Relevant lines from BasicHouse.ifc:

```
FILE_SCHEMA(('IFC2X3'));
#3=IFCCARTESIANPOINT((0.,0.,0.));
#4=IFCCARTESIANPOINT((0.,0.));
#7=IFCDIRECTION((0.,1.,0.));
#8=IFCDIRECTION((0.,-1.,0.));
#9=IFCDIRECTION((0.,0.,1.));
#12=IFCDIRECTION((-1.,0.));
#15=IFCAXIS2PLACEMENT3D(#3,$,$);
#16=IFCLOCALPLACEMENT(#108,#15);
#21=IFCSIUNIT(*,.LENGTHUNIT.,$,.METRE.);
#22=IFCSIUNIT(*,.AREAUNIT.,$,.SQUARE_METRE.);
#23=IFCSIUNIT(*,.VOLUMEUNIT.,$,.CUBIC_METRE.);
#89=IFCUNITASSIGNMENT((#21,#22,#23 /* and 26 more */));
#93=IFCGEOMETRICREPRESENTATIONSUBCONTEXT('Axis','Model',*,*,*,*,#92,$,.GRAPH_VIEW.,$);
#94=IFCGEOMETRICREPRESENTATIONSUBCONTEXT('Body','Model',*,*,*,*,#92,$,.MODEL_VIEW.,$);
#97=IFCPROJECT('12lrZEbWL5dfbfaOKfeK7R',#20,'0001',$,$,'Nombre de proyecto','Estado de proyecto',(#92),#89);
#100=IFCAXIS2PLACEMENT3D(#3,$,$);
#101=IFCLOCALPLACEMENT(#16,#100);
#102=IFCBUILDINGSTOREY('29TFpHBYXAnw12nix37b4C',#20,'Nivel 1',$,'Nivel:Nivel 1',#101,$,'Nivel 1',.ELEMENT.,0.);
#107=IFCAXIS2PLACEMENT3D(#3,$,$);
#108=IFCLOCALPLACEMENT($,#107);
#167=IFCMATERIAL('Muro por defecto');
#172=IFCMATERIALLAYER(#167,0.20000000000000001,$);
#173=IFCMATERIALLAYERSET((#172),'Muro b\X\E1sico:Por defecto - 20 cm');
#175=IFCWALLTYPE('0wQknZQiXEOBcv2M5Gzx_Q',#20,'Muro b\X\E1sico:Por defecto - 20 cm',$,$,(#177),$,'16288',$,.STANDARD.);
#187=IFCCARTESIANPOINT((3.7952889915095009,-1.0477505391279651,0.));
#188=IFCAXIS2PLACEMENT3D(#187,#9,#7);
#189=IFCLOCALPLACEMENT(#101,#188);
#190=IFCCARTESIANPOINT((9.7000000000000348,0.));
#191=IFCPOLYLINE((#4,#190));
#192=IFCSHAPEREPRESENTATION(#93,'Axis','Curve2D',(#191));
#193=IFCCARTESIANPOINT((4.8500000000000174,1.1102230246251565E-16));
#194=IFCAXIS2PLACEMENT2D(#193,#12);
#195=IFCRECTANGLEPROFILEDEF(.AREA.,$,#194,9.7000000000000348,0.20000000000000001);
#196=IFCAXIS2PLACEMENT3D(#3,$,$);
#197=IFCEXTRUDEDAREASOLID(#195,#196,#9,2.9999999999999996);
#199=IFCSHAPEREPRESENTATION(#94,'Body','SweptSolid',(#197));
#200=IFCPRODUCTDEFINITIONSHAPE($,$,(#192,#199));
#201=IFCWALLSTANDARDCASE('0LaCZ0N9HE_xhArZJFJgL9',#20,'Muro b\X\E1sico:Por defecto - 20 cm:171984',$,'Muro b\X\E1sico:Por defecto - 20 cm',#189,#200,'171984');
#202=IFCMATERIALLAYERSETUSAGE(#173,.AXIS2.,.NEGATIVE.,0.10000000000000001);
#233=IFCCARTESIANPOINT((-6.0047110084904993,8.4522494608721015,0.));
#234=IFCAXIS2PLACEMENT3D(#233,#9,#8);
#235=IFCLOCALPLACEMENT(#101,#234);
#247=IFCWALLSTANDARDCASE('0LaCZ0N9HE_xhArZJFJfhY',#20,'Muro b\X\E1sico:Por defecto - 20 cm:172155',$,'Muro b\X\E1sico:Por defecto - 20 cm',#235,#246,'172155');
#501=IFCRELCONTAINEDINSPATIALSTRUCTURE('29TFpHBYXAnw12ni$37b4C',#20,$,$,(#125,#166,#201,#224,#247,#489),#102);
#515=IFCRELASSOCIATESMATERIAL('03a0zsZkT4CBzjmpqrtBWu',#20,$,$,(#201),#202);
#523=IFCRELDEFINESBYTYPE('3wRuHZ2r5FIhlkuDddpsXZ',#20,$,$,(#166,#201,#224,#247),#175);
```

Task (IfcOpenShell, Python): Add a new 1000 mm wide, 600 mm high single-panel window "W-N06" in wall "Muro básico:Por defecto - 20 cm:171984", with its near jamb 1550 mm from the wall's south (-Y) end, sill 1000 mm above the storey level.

```python
import numpy as np
import ifcopenshell
import ifcopenshell.api.feature
import ifcopenshell.api.geometry
import ifcopenshell.api.root
import ifcopenshell.api.spatial
import ifcopenshell.api.type
import ifcopenshell.geom
import ifcopenshell.util.element
import ifcopenshell.util.placement
import ifcopenshell.util.representation
import ifcopenshell.util.shape
import ifcopenshell.util.unit

model = ifcopenshell.open("BasicHouse.ifc")
unit_scale = ifcopenshell.util.unit.calculate_unit_scale(model)
settings = ifcopenshell.geom.settings()


def volume(element):
    """Net volume in cubic metres, openings subtracted."""
    shape = ifcopenshell.geom.create_shape(settings, element)
    return ifcopenshell.util.shape.get_volume(shape.geometry)


wall = model.by_guid("0LaCZ0N9HE_xhArZJFJgL9")
storey = ifcopenshell.util.element.get_container(wall, ifc_class="IfcBuildingStorey")
context = ifcopenshell.util.representation.get_context(model, "Model", "Body", "MODEL_VIEW")
before = volume(wall)

width, height, from_end, sill = 1, 0.6, 1.55, 1  # metres

# The wall runs along its own X axis, and the end named is its -X end.
wall_shape = ifcopenshell.geom.create_shape(settings, wall)
x, y, z = ifcopenshell.util.shape.get_vertices(wall_shape.geometry).T
start = x.min() + from_end
face, thickness = float(y.min()), float(y.max() - y.min())
wall_matrix = ifcopenshell.util.placement.get_local_placement(wall.ObjectPlacement)
level = ifcopenshell.util.placement.get_local_placement(storey.ObjectPlacement)[2, 3]


def in_wall(x, y):
    """Placement at x, y metres in the wall's axes, at sill height."""
    matrix = wall_matrix.copy()
    matrix[:, 3] = wall_matrix @ np.array([x / unit_scale, y / unit_scale, 0.0, 1.0])
    matrix[2, 3] = level + sill / unit_scale
    return matrix


# Opening: a box that overshoots both wall faces by 50 mm.
opening = ifcopenshell.api.root.create_entity(model, ifc_class="IfcOpeningElement")
box = ifcopenshell.api.geometry.add_wall_representation(
    model, context=context, length=width, height=height, thickness=thickness + 0.1
)
ifcopenshell.api.geometry.assign_representation(model, product=opening, representation=box)
ifcopenshell.api.geometry.edit_object_placement(model, product=opening, matrix=in_wall(start, face - 0.05), is_si=False)
ifcopenshell.api.feature.add_feature(model, feature=opening, element=wall)

window = ifcopenshell.api.root.create_entity(model, ifc_class="IfcWindow", name="W-N06")
window.OverallWidth, window.OverallHeight = width / unit_scale, height / unit_scale
body = ifcopenshell.api.geometry.add_window_representation(
    model,
    context=context,
    overall_width=window.OverallWidth,
    overall_height=window.OverallHeight,
    partition_type="SINGLE_PANEL",
)
ifcopenshell.api.geometry.assign_representation(model, product=window, representation=body)
ifcopenshell.api.spatial.assign_container(model, products=[window], relating_structure=storey)
fills = ifcopenshell.api.feature.add_filling(model, opening=opening, element=window)
fills.OwnerHistory = window.OwnerHistory  # required in IFC2X3

# IFC2X3 keeps the operation on the window style.
style = ifcopenshell.api.root.create_entity(model, ifc_class="IfcWindowStyle", name="W-N06")
style.OperationType, style.ConstructionType = "SINGLE_PANEL", "NOTDEFINED"
style.ParameterTakesPrecedence = style.Sizeable = False
ifcopenshell.api.type.assign_type(model, related_objects=[window], relating_type=style)

# Centre the window in the wall's thickness.
ifcopenshell.api.geometry.edit_object_placement(model, product=window, matrix=in_wall(start, face), is_si=False)
window_shape = ifcopenshell.geom.create_shape(settings, window)
depth = ifcopenshell.util.shape.get_vertices(window_shape.geometry)[:, 1]
offset = face + thickness / 2 - (depth.min() + depth.max()) / 2
ifcopenshell.api.geometry.edit_object_placement(model, product=window, matrix=in_wall(start, offset), is_si=False)

after = volume(wall)

print(f"wall volume {before:.3f} -> {after:.3f} m3")

model.write("BasicHouse-out.ifc")
```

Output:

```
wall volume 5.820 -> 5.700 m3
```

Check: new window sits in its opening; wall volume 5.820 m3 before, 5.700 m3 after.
